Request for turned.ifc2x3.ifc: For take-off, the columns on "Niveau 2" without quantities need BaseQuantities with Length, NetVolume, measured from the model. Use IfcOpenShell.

First a look at what the model holds.

```python
import ifcopenshell
import ifcopenshell.util.element
import ifcopenshell.util.unit

model = ifcopenshell.open("turned.ifc2x3.ifc")
print(model.schema)
for unit_type in ("LENGTHUNIT", "AREAUNIT", "VOLUMEUNIT"):
    print(unit_type, ifcopenshell.util.unit.calculate_unit_scale(model, unit_type))
storey = next(s for s in model.by_type("IfcBuildingStorey") if s.Name == "Niveau 2")
columns = [e for e in ifcopenshell.util.element.get_decomposition(storey) if e.is_a("IfcColumn")]
for e in sorted(columns, key=lambda e: e.id()):
    print(e.id(), e.is_a(), e.Name, list(ifcopenshell.util.element.get_psets(e, qtos_only=True)), sep=" | ")
```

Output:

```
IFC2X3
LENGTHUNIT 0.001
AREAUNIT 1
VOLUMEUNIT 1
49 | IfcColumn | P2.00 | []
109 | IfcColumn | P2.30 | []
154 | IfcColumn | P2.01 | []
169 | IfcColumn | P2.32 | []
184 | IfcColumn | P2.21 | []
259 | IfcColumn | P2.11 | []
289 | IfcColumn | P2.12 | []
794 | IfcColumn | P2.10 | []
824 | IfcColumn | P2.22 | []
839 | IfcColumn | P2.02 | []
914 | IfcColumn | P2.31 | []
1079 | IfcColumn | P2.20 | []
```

```python
import ifcopenshell
import ifcopenshell.api.pset
import ifcopenshell.geom
import ifcopenshell.util.element
import ifcopenshell.util.shape
import ifcopenshell.util.unit

model = ifcopenshell.open("turned.ifc2x3.ifc")
unit_scale = ifcopenshell.util.unit.calculate_unit_scale(model)
volume_scale = ifcopenshell.util.unit.calculate_unit_scale(model, "VOLUMEUNIT")
settings = ifcopenshell.geom.settings()

storey = next(s for s in model.by_type("IfcBuildingStorey") if s.Name == "Niveau 2")
columns = [e for e in ifcopenshell.util.element.get_decomposition(storey) if e.is_a("IfcColumn")]

for e in sorted(columns, key=lambda e: e.id()):
    if ifcopenshell.util.element.get_psets(e, qtos_only=True, should_inherit=False):
        continue
    # Geometry comes back in metres, in the element's own axes.
    shape = ifcopenshell.geom.create_shape(settings, e)
    values = {
        "Length": ifcopenshell.util.shape.get_z(shape.geometry) / unit_scale,
        "NetVolume": ifcopenshell.util.shape.get_volume(shape.geometry) / volume_scale,
    }
    qto = ifcopenshell.api.pset.add_qto(model, product=e, name="BaseQuantities")
    ifcopenshell.api.pset.edit_qto(model, qto=qto, properties=values)
    print(e.id(), {k: round(v, 3) for k, v in values.items()})

model.write("turned.ifc2x3_rev.ifc")
```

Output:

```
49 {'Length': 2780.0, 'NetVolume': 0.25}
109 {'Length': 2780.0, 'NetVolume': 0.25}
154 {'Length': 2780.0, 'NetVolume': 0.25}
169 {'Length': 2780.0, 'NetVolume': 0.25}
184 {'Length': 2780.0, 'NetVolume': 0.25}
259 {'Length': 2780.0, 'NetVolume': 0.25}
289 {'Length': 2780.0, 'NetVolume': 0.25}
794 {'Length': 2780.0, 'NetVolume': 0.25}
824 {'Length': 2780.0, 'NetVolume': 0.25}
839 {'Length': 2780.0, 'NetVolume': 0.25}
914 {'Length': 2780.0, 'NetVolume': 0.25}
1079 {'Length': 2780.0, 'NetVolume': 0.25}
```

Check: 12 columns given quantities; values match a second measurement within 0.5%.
